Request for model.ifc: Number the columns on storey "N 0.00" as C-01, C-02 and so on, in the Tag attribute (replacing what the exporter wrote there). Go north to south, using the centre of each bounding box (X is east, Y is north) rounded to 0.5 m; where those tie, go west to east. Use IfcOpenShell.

First a look at what the model holds.

```python
import ifcopenshell
import ifcopenshell.util.element
import ifcopenshell.util.placement

model = ifcopenshell.open("model.ifc")
print(model.schema)
storey = next(s for s in model.by_type("IfcBuildingStorey") if s.Name == "N 0.00")
columns = [e for e in ifcopenshell.util.element.get_decomposition(storey) if e.is_a("IfcColumn")]
for e in sorted(columns, key=lambda e: e.id()):
    origin = ifcopenshell.util.placement.get_local_placement(e.ObjectPlacement)[:3, 3]
    print(e.id(), e.Tag, e.Name, origin.round(2) + 0.0, sep=" | ")
```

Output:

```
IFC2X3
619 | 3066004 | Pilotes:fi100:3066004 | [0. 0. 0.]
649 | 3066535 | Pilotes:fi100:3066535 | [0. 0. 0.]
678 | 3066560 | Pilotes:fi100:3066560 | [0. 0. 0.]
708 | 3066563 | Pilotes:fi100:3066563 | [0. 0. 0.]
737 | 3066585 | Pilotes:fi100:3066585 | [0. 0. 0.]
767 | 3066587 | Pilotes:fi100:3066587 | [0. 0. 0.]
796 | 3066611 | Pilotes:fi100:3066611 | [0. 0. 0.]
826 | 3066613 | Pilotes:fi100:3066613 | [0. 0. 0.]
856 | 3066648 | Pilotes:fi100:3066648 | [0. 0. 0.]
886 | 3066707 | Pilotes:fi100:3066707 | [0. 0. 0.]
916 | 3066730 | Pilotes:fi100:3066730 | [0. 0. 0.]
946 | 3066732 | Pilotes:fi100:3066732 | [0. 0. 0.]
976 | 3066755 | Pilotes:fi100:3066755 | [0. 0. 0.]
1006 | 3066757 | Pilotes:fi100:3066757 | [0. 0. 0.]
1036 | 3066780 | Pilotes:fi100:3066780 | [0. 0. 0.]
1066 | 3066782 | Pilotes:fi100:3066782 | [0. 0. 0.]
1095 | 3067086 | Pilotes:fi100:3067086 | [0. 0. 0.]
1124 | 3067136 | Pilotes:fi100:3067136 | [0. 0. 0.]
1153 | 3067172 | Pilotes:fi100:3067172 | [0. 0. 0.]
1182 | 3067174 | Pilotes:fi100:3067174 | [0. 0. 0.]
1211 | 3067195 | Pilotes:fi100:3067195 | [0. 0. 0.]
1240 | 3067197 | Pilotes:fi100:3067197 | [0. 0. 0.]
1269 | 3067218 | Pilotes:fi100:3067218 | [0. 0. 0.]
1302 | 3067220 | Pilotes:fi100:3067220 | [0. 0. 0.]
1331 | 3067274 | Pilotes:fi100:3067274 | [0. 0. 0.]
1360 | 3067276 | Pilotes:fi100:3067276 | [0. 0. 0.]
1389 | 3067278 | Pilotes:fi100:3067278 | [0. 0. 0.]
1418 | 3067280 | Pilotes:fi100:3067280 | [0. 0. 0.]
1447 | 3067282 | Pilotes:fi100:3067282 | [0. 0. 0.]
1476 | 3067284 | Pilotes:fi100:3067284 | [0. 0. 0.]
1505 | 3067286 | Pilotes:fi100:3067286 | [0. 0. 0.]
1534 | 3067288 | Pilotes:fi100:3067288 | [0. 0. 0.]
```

```python
import ifcopenshell
import ifcopenshell.geom
import ifcopenshell.util.element
import ifcopenshell.util.shape

model = ifcopenshell.open("model.ifc")
settings = ifcopenshell.geom.settings()
settings.set("use-world-coords", True)


def centre(element):
    shape = ifcopenshell.geom.create_shape(settings, element)
    return ifcopenshell.util.shape.get_bbox_centroid(shape.geometry)


storey = next(s for s in model.by_type("IfcBuildingStorey") if s.Name == "N 0.00")
columns = [e for e in ifcopenshell.util.element.get_decomposition(storey) if e.is_a("IfcColumn")]

# Insertion points can sit at a corner or the storey origin, so sort by the geometry (in metres).
centres = {e: centre(e) for e in columns}
columns.sort(key=lambda e: (-round(centres[e][1] / 0.5), centres[e][0]))

for i, e in enumerate(columns, start=1):
    number = f"C-{i:02d}"
    e.Tag = number
    print(e.id(), number)

model.write("model_edited.ifc")
```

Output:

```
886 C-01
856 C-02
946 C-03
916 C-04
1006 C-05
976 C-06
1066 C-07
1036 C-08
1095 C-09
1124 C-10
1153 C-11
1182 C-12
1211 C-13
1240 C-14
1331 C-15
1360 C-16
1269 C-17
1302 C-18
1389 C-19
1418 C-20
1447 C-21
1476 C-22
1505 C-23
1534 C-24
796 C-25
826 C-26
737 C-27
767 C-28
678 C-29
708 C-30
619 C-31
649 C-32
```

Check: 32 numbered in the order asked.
